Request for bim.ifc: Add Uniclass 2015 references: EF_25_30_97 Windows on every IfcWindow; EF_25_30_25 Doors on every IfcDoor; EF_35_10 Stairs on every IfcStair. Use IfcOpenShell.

First a look at what the model holds.

```python
import ifcopenshell

model = ifcopenshell.open("bim.ifc")
print(model.schema)
print("classifications:", [c.Name for c in model.by_type("IfcClassification")])
for ifc_class in ("IfcDoor", "IfcRoof", "IfcStair", "IfcWall", "IfcWindow"):
    print(ifc_class, len(model.by_type(ifc_class)))
```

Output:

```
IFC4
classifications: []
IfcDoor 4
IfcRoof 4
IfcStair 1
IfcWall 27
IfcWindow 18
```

```python
import ifcopenshell
import ifcopenshell.api.classification

model = ifcopenshell.open("bim.ifc")

system = ifcopenshell.api.classification.add_classification(model, classification="Uniclass 2015")

codes = {
    "IfcWindow": ("EF_25_30_97", "Windows"),
    "IfcDoor": ("EF_25_30_25", "Doors"),
    "IfcStair": ("EF_35_10", "Stairs"),
}
for ifc_class, (code, name) in codes.items():
    products = model.by_type(ifc_class)
    ifcopenshell.api.classification.add_reference(
        model, products=products, classification=system, identification=code, name=name
    )
    print(code, len(products))

model.write("bim_updated.ifc")
```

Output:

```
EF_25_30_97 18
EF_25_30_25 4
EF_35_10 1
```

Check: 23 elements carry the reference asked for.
